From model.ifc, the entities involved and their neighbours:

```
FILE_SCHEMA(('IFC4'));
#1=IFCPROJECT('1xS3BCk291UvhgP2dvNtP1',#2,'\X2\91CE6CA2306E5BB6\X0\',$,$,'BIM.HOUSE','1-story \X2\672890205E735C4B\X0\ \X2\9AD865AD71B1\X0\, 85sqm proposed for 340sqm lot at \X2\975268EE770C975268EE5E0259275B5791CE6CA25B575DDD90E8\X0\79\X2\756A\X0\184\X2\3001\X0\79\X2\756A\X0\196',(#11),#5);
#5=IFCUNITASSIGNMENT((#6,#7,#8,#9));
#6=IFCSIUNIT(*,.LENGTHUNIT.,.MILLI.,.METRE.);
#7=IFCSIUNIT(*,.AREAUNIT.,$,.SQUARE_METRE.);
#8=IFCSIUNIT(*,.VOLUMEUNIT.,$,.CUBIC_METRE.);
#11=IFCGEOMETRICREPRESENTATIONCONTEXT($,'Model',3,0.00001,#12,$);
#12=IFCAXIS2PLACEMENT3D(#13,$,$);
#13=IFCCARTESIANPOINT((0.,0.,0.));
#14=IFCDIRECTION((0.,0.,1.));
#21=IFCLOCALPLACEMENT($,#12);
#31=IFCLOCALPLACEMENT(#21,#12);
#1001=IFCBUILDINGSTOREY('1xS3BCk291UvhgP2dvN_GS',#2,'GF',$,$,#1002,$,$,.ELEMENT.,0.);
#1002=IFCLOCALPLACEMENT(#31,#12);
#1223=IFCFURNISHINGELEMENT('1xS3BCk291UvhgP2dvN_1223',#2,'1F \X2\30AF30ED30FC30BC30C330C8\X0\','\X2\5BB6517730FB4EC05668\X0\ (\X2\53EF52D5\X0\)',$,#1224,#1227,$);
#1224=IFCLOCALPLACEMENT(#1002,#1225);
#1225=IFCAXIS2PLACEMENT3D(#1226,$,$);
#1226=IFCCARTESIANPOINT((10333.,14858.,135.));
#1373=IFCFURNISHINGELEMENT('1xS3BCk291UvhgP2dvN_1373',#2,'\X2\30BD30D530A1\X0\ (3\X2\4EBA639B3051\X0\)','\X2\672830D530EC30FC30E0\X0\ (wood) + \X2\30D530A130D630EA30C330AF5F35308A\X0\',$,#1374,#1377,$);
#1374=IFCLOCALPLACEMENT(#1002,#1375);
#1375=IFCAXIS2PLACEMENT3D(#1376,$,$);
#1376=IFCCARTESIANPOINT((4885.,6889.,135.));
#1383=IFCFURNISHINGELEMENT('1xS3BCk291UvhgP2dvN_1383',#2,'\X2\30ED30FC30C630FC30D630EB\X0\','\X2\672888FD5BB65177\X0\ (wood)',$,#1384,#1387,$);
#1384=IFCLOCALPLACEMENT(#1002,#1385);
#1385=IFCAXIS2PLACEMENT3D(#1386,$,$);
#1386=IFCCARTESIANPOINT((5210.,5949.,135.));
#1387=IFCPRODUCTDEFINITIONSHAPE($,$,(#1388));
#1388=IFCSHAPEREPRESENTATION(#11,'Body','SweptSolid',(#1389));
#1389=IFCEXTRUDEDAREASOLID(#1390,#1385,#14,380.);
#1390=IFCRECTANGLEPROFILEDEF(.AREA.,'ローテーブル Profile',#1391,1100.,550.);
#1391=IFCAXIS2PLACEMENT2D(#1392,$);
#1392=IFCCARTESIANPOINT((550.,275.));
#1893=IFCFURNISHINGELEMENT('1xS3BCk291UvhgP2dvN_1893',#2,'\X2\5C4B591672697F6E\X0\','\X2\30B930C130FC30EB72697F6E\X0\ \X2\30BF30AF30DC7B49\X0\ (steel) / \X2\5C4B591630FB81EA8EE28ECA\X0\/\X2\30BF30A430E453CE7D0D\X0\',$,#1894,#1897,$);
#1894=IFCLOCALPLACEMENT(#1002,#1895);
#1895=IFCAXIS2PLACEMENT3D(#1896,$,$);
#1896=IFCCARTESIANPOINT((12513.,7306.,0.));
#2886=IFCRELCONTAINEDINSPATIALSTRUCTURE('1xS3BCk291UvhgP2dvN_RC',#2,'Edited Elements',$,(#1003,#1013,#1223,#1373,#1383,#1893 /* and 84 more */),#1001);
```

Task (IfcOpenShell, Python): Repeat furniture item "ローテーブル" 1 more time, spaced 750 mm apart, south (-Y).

```python
import numpy as np
import ifcopenshell
import ifcopenshell.api.geometry
import ifcopenshell.api.root
import ifcopenshell.util.element
import ifcopenshell.util.placement
import ifcopenshell.util.unit

model = ifcopenshell.open("model.ifc")
unit_scale = ifcopenshell.util.unit.calculate_unit_scale(model)


def reuse_history(source, copy):
    """copy_class also copies each property set's owner history, people and application; keep the originals."""
    for rel in copy.IsDefinedBy:
        if rel.is_a("IfcRelDefinesByProperties") and (history := rel.RelatingPropertyDefinition.OwnerHistory):
            rel.RelatingPropertyDefinition.OwnerHistory = source.OwnerHistory
            ifcopenshell.util.element.remove_deep2(model, history)


source = model.by_guid("1xS3BCk291UvhgP2dvN_1383")
base = ifcopenshell.util.placement.get_local_placement(source.ObjectPlacement)
step = np.array([0.0, -1.0, 0.0]) * 0.75 / unit_scale

for i in range(1, 2):
    copy = ifcopenshell.api.root.copy_class(model, product=source)
    copy.Representation = ifcopenshell.util.element.copy_deep(
        model, source.Representation, exclude=["IfcGeometricRepresentationContext", "IfcRepresentationMap"]
    )
    reuse_history(source, copy)
    matrix = base.copy()
    matrix[:3, 3] += i * step
    print("added at", matrix[:3, 3].round(3) + 0.0)
    ifcopenshell.api.geometry.edit_object_placement(model, product=copy, matrix=matrix, is_si=False)

model.write("model-out.ifc")
```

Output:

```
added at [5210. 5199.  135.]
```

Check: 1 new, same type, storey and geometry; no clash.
